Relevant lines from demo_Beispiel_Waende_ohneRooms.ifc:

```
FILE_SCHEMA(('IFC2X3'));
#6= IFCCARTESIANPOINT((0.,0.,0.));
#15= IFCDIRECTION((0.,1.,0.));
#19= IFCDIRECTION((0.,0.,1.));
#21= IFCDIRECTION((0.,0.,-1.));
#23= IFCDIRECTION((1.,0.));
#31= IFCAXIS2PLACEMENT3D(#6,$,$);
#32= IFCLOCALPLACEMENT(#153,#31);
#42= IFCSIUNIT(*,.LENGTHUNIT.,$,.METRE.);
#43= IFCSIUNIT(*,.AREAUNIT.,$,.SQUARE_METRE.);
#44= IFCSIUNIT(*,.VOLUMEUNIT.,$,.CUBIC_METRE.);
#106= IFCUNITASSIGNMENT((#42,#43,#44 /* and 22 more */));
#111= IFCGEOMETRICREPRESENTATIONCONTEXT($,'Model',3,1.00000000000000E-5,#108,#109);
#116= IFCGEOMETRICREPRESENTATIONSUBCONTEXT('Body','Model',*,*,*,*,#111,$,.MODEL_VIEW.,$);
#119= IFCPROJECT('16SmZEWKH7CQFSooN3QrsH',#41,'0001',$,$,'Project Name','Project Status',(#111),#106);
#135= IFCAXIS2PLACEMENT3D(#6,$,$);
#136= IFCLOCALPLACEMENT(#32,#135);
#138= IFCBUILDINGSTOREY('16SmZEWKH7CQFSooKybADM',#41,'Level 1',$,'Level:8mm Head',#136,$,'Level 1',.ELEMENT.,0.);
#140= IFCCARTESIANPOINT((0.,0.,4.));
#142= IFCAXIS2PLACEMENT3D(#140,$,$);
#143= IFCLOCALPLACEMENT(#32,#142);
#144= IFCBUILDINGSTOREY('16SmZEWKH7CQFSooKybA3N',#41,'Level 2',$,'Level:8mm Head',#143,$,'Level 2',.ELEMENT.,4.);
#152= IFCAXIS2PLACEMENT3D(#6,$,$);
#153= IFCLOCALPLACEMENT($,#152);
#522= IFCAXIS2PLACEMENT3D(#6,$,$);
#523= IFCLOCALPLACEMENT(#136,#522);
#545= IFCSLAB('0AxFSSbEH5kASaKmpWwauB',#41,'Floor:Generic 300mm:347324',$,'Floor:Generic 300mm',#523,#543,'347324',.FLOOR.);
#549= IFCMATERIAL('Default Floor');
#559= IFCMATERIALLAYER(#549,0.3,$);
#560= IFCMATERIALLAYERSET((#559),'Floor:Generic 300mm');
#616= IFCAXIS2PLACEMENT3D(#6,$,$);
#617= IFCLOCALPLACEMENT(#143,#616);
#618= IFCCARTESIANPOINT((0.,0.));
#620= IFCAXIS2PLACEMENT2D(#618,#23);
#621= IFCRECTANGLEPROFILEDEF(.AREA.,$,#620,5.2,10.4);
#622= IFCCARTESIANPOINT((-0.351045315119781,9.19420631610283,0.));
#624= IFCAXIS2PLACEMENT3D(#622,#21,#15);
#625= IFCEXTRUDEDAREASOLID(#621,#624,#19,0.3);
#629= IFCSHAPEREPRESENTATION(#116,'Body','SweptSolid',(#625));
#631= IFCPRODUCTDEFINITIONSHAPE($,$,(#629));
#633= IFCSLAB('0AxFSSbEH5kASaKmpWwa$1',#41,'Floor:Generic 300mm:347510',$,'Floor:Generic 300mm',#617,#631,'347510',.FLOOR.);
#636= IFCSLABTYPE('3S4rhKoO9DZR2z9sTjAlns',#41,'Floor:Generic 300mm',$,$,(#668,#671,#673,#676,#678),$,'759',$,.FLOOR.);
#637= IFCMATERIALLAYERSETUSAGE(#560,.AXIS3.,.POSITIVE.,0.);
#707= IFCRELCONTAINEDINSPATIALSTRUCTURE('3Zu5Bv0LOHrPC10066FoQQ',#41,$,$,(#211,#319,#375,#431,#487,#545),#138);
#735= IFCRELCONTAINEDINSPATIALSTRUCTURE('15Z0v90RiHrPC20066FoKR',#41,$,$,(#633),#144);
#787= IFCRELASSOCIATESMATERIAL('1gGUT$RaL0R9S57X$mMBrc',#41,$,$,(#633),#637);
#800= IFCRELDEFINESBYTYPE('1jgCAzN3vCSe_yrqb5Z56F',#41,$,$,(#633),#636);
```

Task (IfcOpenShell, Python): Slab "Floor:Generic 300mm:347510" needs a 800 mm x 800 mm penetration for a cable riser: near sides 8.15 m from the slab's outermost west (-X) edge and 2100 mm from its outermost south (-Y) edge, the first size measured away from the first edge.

```python
import numpy as np
import ifcopenshell
import ifcopenshell.api.feature
import ifcopenshell.api.geometry
import ifcopenshell.api.root
import ifcopenshell.geom
import ifcopenshell.util.placement
import ifcopenshell.util.representation
import ifcopenshell.util.shape
import ifcopenshell.util.unit

model = ifcopenshell.open("demo_Beispiel_Waende_ohneRooms.ifc")
unit_scale = ifcopenshell.util.unit.calculate_unit_scale(model)
settings = ifcopenshell.geom.settings()


def volume(element):
    """Net volume in cubic metres, openings subtracted."""
    shape = ifcopenshell.geom.create_shape(settings, element)
    return ifcopenshell.util.shape.get_volume(shape.geometry)


slab = model.by_guid("0AxFSSbEH5kASaKmpWwa$1")
before = volume(slab)

# Extent in the slab's own axes, in metres. The edges named are its -X and -Y sides.
slab_shape = ifcopenshell.geom.create_shape(settings, slab)
vertices = ifcopenshell.util.shape.get_vertices(slab_shape.geometry)
x_min, y_min, bottom = vertices.min(axis=0)
top = vertices[:, 2].max()

opening = ifcopenshell.api.root.create_entity(model, ifc_class="IfcOpeningElement", name="Cable riser opening")
context = ifcopenshell.util.representation.get_context(model, "Model", "Body", "MODEL_VIEW")
width, depth = 0.8, 0.8
outline = [(0.0, 0.0), (width, 0.0), (width, depth), (0.0, depth), (0.0, 0.0)]
# Overshoot both faces by 50 mm so the cut is clean.
shape = ifcopenshell.api.geometry.add_slab_representation(
    model, context=context, depth=top - bottom + 0.1, polyline=outline
)
ifcopenshell.api.geometry.assign_representation(model, product=opening, representation=shape)

matrix = ifcopenshell.util.placement.get_local_placement(slab.ObjectPlacement)
matrix[:, 3] = matrix @ np.append(np.array([x_min + 8.15, y_min + 2.1, bottom - 0.05]) / unit_scale, 1.0)
ifcopenshell.api.geometry.edit_object_placement(model, product=opening, matrix=matrix, is_si=False)
ifcopenshell.api.feature.add_feature(model, feature=opening, element=slab)

after = volume(slab)

print(f"slab volume {before:.3f} -> {after:.3f} m3")

model.write("demo_Beispiel_Waende_ohneRooms-out.ifc")
```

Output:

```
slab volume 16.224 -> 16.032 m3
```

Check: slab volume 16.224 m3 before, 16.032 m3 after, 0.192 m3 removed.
